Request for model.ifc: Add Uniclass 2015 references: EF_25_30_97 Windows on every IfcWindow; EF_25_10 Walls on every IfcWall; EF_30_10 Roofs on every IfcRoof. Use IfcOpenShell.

First a look at what the model holds.

```python
import ifcopenshell

model = ifcopenshell.open("model.ifc")
print(model.schema)
print("classifications:", [c.Name for c in model.by_type("IfcClassification")])
for ifc_class in ("IfcDoor", "IfcRoof", "IfcStair", "IfcWall", "IfcWindow"):
    print(ifc_class, len(model.by_type(ifc_class)))
```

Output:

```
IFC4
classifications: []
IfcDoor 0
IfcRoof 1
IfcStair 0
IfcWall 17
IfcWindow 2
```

```python
import ifcopenshell
import ifcopenshell.api.classification

model = ifcopenshell.open("model.ifc")

system = ifcopenshell.api.classification.add_classification(model, classification="Uniclass 2015")

codes = {
    "IfcWindow": ("EF_25_30_97", "Windows"),
    "IfcWall": ("EF_25_10", "Walls"),
    "IfcRoof": ("EF_30_10", "Roofs"),
}
for ifc_class, (code, name) in codes.items():
    products = model.by_type(ifc_class)
    ifcopenshell.api.classification.add_reference(
        model, products=products, classification=system, identification=code, name=name
    )
    print(code, len(products))

model.write("model_v2.ifc")
```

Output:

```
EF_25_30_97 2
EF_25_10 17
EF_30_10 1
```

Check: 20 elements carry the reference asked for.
